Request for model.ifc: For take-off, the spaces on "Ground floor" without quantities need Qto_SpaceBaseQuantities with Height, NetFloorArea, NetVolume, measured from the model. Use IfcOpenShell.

First a look at what the model holds.

```python
import ifcopenshell
import ifcopenshell.util.element
import ifcopenshell.util.unit

model = ifcopenshell.open("model.ifc")
print(model.schema)
for unit_type in ("LENGTHUNIT", "AREAUNIT", "VOLUMEUNIT"):
    print(unit_type, ifcopenshell.util.unit.calculate_unit_scale(model, unit_type))
storey = next(s for s in model.by_type("IfcBuildingStorey") if s.Name == "Ground floor")
spaces = [e for e in ifcopenshell.util.element.get_decomposition(storey) if e.is_a("IfcSpace")]
for e in sorted(spaces, key=lambda e: e.id()):
    print(e.id(), e.is_a(), e.Name, list(ifcopenshell.util.element.get_psets(e, qtos_only=True)), sep=" | ")
```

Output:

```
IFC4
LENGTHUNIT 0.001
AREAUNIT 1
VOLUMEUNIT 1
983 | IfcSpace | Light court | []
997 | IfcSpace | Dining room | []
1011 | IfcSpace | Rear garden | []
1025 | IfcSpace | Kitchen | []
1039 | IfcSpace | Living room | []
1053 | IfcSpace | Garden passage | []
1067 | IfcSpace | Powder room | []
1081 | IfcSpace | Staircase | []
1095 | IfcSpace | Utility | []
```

```python
import ifcopenshell
import ifcopenshell.api.pset
import ifcopenshell.geom
import ifcopenshell.util.element
import ifcopenshell.util.shape
import ifcopenshell.util.unit

model = ifcopenshell.open("model.ifc")
unit_scale = ifcopenshell.util.unit.calculate_unit_scale(model)
area_scale = ifcopenshell.util.unit.calculate_unit_scale(model, "AREAUNIT")
volume_scale = ifcopenshell.util.unit.calculate_unit_scale(model, "VOLUMEUNIT")
settings = ifcopenshell.geom.settings()

storey = next(s for s in model.by_type("IfcBuildingStorey") if s.Name == "Ground floor")
spaces = [e for e in ifcopenshell.util.element.get_decomposition(storey) if e.is_a("IfcSpace")]

for e in sorted(spaces, key=lambda e: e.id()):
    if ifcopenshell.util.element.get_psets(e, qtos_only=True, should_inherit=False):
        continue
    # Geometry comes back in metres, in the element's own axes.
    shape = ifcopenshell.geom.create_shape(settings, e)
    values = {
        "Height": ifcopenshell.util.shape.get_z(shape.geometry) / unit_scale,
        "NetFloorArea": ifcopenshell.util.shape.get_footprint_area(shape.geometry) / area_scale,
        "NetVolume": ifcopenshell.util.shape.get_volume(shape.geometry) / volume_scale,
    }
    qto = ifcopenshell.api.pset.add_qto(model, product=e, name="Qto_SpaceBaseQuantities")
    ifcopenshell.api.pset.edit_qto(model, qto=qto, properties=values)
    print(e.id(), {k: round(v, 3) for k, v in values.items()})

model.write("model-out.ifc")
```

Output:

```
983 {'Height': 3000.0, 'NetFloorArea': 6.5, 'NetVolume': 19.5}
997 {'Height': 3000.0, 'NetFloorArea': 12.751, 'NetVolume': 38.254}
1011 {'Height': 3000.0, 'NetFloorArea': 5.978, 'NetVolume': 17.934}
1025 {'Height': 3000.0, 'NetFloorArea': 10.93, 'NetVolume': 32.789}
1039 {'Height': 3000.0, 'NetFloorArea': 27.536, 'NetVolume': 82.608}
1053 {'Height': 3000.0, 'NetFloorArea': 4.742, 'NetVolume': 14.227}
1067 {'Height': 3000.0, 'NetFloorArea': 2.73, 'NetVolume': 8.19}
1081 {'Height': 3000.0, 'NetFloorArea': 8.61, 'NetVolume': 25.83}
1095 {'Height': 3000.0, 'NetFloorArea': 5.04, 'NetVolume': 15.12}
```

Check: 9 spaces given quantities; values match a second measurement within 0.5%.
